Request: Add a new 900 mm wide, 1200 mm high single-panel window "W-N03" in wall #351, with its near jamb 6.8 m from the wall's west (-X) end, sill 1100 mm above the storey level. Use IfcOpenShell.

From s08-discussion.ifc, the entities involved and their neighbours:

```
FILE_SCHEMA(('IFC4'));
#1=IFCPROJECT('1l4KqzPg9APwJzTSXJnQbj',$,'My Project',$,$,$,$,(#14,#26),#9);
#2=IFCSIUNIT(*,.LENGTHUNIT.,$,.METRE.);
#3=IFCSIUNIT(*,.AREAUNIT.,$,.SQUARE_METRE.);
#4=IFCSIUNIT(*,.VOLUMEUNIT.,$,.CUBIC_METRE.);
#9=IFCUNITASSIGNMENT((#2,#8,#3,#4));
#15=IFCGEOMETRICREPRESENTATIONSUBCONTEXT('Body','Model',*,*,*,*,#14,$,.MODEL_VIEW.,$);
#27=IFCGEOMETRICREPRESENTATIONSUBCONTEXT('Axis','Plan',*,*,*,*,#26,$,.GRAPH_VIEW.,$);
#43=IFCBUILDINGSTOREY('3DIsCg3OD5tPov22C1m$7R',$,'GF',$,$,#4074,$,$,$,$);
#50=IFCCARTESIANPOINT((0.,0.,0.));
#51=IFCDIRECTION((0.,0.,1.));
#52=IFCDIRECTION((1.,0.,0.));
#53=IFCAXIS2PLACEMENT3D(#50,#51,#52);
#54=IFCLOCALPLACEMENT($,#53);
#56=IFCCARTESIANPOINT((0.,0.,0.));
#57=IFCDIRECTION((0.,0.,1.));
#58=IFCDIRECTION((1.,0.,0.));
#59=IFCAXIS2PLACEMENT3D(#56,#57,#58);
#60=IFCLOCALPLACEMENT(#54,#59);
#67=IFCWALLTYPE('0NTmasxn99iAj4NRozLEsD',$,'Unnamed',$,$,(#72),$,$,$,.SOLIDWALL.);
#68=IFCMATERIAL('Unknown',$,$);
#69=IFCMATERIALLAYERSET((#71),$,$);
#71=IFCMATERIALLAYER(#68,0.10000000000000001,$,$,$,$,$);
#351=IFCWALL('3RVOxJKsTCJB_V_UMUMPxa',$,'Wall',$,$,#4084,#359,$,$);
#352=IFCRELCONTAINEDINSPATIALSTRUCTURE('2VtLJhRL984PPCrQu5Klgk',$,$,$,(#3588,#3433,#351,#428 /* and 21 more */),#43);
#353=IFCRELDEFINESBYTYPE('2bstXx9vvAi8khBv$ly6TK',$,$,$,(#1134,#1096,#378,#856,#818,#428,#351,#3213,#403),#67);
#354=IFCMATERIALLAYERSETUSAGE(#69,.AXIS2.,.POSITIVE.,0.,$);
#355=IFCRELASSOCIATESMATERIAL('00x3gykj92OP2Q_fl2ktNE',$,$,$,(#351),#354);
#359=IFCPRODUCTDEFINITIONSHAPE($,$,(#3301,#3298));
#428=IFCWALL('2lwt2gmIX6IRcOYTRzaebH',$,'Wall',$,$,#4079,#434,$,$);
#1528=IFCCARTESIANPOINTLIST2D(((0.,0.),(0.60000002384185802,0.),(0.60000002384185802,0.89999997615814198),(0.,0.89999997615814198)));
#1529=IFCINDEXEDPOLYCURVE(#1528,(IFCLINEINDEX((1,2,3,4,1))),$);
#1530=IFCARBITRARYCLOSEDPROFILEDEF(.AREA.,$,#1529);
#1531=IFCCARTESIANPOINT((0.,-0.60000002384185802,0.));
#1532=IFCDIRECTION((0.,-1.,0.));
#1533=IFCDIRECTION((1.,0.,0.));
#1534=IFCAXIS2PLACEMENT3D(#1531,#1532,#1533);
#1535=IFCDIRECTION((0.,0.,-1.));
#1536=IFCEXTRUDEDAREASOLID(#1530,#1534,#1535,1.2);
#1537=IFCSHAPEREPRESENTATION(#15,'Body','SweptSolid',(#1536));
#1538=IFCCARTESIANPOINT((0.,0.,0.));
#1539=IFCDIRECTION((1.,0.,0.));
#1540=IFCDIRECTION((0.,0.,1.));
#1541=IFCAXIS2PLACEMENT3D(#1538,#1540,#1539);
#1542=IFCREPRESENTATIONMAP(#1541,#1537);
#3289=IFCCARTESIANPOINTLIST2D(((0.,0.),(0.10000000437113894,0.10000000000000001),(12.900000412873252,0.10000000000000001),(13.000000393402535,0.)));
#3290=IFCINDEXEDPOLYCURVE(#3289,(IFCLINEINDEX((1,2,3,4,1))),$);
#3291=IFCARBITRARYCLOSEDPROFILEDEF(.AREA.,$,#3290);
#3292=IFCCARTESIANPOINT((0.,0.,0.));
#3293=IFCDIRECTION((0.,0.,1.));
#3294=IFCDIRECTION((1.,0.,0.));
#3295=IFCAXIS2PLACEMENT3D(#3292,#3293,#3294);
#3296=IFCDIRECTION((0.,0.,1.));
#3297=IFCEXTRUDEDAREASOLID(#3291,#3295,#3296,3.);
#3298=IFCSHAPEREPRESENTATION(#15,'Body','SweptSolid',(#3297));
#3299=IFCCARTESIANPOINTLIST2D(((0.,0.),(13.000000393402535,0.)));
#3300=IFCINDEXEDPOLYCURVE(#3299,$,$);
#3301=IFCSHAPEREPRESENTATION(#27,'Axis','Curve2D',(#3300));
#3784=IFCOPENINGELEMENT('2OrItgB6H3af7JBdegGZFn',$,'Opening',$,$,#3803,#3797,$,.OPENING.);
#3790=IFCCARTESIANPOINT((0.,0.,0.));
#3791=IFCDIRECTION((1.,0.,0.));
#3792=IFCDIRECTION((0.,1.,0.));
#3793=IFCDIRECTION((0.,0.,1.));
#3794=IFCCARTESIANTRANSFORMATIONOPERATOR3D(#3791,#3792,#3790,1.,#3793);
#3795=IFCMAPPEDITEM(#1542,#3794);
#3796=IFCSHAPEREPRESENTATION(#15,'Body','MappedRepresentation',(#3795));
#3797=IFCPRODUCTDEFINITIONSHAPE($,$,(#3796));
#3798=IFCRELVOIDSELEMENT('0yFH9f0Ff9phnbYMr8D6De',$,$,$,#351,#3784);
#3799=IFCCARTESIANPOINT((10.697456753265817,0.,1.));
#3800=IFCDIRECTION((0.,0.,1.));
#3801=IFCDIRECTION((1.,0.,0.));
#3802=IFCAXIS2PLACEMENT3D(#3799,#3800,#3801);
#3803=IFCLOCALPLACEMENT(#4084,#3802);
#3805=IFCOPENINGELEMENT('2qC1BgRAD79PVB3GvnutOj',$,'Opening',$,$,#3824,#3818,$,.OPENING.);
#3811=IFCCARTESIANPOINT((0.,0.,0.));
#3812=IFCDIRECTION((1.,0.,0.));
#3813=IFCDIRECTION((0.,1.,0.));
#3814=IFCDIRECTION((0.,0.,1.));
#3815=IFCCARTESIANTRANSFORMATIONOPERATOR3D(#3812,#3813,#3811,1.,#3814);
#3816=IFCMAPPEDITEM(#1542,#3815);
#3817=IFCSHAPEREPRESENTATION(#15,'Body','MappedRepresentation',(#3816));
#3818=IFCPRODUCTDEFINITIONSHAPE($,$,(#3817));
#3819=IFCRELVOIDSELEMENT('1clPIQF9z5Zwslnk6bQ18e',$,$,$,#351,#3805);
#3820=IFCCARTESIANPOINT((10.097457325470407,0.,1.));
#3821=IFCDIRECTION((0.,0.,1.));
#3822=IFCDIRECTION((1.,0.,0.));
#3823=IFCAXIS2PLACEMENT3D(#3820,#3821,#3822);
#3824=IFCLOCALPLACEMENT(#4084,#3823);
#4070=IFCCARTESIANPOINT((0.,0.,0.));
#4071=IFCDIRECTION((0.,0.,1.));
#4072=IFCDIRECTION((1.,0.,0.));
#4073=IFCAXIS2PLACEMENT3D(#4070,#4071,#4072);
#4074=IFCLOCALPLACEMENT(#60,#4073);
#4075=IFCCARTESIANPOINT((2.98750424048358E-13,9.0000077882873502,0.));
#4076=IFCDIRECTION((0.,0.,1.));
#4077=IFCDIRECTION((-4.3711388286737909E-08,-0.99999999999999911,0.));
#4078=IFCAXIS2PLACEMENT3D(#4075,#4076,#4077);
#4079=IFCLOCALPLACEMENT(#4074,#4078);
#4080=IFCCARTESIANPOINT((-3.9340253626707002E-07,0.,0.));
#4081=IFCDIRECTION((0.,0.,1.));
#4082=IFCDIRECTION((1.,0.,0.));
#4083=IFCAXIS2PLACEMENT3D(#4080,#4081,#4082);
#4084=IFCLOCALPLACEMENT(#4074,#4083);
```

```python
import numpy as np
import ifcopenshell
import ifcopenshell.api.feature
import ifcopenshell.api.geometry
import ifcopenshell.api.root
import ifcopenshell.api.spatial
import ifcopenshell.geom
import ifcopenshell.util.element
import ifcopenshell.util.placement
import ifcopenshell.util.representation
import ifcopenshell.util.shape
import ifcopenshell.util.unit

model = ifcopenshell.open("s08-discussion.ifc")
unit_scale = ifcopenshell.util.unit.calculate_unit_scale(model)
settings = ifcopenshell.geom.settings()


def volume(element):
    """Net volume in cubic metres, openings subtracted."""
    shape = ifcopenshell.geom.create_shape(settings, element)
    return ifcopenshell.util.shape.get_volume(shape.geometry)


wall = model.by_id(351)
storey = ifcopenshell.util.element.get_container(wall, ifc_class="IfcBuildingStorey")
context = ifcopenshell.util.representation.get_context(model, "Model", "Body", "MODEL_VIEW")
before = volume(wall)

width, height, from_end, sill = 0.9, 1.2, 6.8, 1.1  # metres

# The wall runs along its own X axis, and the end named is its -X end.
wall_shape = ifcopenshell.geom.create_shape(settings, wall)
x, y, z = ifcopenshell.util.shape.get_vertices(wall_shape.geometry).T
start = x.min() + from_end
face, thickness = float(y.min()), float(y.max() - y.min())
wall_matrix = ifcopenshell.util.placement.get_local_placement(wall.ObjectPlacement)
level = ifcopenshell.util.placement.get_local_placement(storey.ObjectPlacement)[2, 3]


def in_wall(x, y):
    """Placement at x, y metres in the wall's axes, at sill height."""
    matrix = wall_matrix.copy()
    matrix[:, 3] = wall_matrix @ np.array([x / unit_scale, y / unit_scale, 0.0, 1.0])
    matrix[2, 3] = level + sill / unit_scale
    return matrix


# Opening: a box that overshoots both wall faces by 50 mm.
opening = ifcopenshell.api.root.create_entity(model, ifc_class="IfcOpeningElement", predefined_type="OPENING")
box = ifcopenshell.api.geometry.add_wall_representation(
    model, context=context, length=width, height=height, thickness=thickness + 0.1
)
ifcopenshell.api.geometry.assign_representation(model, product=opening, representation=box)
ifcopenshell.api.geometry.edit_object_placement(model, product=opening, matrix=in_wall(start, face - 0.05), is_si=False)
ifcopenshell.api.feature.add_feature(model, feature=opening, element=wall)

window = ifcopenshell.api.root.create_entity(model, ifc_class="IfcWindow", name="W-N03", predefined_type="WINDOW")
window.OverallWidth, window.OverallHeight = width / unit_scale, height / unit_scale
window.PartitioningType = "SINGLE_PANEL"
body = ifcopenshell.api.geometry.add_window_representation(
    model,
    context=context,
    overall_width=window.OverallWidth,
    overall_height=window.OverallHeight,
    partition_type="SINGLE_PANEL",
)
ifcopenshell.api.geometry.assign_representation(model, product=window, representation=body)
ifcopenshell.api.spatial.assign_container(model, products=[window], relating_structure=storey)
ifcopenshell.api.feature.add_filling(model, opening=opening, element=window)

# Centre the window in the wall's thickness.
ifcopenshell.api.geometry.edit_object_placement(model, product=window, matrix=in_wall(start, face), is_si=False)
window_shape = ifcopenshell.geom.create_shape(settings, window)
depth = ifcopenshell.util.shape.get_vertices(window_shape.geometry)[:, 1]
offset = face + thickness / 2 - (depth.min() + depth.max()) / 2
ifcopenshell.api.geometry.edit_object_placement(model, product=window, matrix=in_wall(start, offset), is_si=False)

after = volume(wall)

print(f"wall volume {before:.3f} -> {after:.3f} m3")

model.write("s08-discussion_edited.ifc")
```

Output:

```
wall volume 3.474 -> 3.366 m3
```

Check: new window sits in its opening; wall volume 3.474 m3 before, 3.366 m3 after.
